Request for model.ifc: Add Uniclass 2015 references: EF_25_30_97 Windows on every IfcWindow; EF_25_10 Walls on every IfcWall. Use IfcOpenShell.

First a look at what the model holds.

```python
import ifcopenshell

model = ifcopenshell.open("model.ifc")
print(model.schema)
print("classifications:", [c.Name for c in model.by_type("IfcClassification")])
for ifc_class in ("IfcDoor", "IfcRoof", "IfcStair", "IfcWall", "IfcWindow"):
    print(ifc_class, len(model.by_type(ifc_class)))
```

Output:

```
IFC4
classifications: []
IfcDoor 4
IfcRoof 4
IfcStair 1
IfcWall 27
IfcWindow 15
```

```python
import ifcopenshell
import ifcopenshell.api.classification

model = ifcopenshell.open("model.ifc")

system = ifcopenshell.api.classification.add_classification(model, classification="Uniclass 2015")

codes = {
    "IfcWindow": ("EF_25_30_97", "Windows"),
    "IfcWall": ("EF_25_10", "Walls"),
}
for ifc_class, (code, name) in codes.items():
    products = model.by_type(ifc_class)
    ifcopenshell.api.classification.add_reference(
        model, products=products, classification=system, identification=code, name=name
    )
    print(code, len(products))

model.write("model-out.ifc")
```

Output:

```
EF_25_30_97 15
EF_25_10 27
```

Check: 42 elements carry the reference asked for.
